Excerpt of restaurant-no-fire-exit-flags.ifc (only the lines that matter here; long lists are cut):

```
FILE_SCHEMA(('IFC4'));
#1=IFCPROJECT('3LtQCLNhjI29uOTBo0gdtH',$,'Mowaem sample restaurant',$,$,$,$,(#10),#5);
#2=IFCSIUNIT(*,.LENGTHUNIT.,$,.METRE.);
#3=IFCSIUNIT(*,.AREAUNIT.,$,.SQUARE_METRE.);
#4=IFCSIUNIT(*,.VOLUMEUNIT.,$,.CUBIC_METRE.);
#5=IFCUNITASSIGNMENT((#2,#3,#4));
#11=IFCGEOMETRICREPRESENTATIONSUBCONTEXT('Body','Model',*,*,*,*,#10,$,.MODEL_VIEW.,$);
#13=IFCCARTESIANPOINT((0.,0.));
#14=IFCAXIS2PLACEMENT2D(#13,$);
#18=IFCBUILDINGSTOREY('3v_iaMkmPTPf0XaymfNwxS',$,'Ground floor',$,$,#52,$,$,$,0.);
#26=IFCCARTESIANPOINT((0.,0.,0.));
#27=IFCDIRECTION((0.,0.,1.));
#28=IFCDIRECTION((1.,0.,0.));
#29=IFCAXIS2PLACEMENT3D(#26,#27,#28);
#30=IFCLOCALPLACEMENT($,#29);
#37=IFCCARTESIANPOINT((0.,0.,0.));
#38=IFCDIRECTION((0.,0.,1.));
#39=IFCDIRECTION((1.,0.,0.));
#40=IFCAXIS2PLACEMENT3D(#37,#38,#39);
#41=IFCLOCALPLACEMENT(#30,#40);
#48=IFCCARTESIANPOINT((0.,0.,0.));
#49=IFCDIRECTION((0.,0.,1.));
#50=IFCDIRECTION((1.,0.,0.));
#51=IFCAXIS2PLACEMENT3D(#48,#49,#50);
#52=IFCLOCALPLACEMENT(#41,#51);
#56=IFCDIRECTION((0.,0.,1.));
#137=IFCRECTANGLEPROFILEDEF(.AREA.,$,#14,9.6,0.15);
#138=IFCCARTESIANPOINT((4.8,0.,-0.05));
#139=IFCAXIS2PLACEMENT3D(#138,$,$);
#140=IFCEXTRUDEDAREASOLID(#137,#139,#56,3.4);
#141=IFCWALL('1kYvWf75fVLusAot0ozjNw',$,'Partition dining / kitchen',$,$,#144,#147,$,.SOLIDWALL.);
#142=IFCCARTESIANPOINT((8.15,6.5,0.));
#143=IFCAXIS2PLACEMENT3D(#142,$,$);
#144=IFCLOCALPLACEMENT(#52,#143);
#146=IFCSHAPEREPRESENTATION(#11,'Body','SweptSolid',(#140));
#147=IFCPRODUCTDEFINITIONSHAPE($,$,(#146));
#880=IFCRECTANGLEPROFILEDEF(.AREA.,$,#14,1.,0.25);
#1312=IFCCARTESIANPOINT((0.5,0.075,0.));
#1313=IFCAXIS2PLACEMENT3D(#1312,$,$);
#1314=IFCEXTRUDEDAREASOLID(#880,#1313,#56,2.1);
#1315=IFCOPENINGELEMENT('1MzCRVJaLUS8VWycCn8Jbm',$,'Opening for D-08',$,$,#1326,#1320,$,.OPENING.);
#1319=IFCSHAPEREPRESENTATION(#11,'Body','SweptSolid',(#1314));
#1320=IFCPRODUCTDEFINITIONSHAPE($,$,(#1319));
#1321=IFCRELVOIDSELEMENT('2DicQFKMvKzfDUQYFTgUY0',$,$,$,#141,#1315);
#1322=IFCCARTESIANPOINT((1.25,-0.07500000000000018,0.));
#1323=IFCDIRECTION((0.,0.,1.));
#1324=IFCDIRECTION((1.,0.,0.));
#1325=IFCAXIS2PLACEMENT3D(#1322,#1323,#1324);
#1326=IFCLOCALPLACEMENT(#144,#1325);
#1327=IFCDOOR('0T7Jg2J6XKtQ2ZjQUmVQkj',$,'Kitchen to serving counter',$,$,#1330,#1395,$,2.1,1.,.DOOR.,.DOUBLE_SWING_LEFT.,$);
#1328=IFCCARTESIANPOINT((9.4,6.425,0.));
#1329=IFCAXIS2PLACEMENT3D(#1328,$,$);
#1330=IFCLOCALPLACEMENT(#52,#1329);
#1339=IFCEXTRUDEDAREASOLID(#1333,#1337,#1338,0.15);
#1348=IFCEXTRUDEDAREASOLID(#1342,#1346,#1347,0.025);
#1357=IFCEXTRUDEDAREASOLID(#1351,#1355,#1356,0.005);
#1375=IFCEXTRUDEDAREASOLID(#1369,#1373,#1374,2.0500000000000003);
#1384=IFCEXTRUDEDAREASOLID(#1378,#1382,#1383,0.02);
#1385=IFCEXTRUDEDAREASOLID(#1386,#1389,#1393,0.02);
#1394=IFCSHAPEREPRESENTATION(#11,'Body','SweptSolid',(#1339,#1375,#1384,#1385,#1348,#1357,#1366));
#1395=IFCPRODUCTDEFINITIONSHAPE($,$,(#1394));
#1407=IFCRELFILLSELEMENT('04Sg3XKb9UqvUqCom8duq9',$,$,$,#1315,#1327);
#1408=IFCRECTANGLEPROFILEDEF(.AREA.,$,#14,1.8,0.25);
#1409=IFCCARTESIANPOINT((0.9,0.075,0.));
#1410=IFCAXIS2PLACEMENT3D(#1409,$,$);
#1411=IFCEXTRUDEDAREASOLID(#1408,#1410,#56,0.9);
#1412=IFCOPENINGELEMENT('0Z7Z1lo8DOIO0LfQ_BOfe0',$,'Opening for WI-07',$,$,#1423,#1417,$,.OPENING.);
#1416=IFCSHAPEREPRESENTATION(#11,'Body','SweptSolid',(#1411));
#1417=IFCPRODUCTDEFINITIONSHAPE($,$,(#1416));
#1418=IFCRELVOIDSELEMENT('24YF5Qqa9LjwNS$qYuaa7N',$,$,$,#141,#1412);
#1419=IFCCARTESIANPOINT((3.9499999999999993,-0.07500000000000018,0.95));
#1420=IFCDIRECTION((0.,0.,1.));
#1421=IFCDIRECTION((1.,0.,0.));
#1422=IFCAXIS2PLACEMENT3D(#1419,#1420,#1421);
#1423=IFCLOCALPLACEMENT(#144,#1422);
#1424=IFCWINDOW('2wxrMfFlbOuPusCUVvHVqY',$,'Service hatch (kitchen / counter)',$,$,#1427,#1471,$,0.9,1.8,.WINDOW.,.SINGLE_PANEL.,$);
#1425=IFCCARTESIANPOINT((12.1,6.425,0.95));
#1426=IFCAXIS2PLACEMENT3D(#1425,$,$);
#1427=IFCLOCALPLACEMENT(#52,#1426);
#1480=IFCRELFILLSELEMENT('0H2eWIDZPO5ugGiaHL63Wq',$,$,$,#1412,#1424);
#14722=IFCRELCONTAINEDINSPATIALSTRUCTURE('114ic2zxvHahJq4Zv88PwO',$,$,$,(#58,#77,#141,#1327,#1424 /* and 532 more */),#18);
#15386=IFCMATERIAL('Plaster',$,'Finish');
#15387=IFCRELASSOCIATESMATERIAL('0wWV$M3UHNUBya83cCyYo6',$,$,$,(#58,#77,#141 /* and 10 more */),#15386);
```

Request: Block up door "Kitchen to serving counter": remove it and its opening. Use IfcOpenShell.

```python
import ifcopenshell
import ifcopenshell.api.feature
import ifcopenshell.api.root
import ifcopenshell.geom
import ifcopenshell.util.shape

model = ifcopenshell.open("restaurant-no-fire-exit-flags.ifc")
settings = ifcopenshell.geom.settings()


def volume(element):
    """Net volume in cubic metres, openings subtracted."""
    shape = ifcopenshell.geom.create_shape(settings, element)
    return ifcopenshell.util.shape.get_volume(shape.geometry)


door = model.by_guid("0T7Jg2J6XKtQ2ZjQUmVQkj")
opening = door.FillsVoids[0].RelatingOpeningElement
wall = opening.VoidsElements[0].RelatingBuildingElement
before = volume(wall)

ifcopenshell.api.root.remove_product(model, product=door)
ifcopenshell.api.feature.remove_feature(model, feature=opening)

after = volume(wall)

print(f"wall volume {before:.3f} -> {after:.3f} m3")

model.write("restaurant-no-fire-exit-flags-out.ifc")
```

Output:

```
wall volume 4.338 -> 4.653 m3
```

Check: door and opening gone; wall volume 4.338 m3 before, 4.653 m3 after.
